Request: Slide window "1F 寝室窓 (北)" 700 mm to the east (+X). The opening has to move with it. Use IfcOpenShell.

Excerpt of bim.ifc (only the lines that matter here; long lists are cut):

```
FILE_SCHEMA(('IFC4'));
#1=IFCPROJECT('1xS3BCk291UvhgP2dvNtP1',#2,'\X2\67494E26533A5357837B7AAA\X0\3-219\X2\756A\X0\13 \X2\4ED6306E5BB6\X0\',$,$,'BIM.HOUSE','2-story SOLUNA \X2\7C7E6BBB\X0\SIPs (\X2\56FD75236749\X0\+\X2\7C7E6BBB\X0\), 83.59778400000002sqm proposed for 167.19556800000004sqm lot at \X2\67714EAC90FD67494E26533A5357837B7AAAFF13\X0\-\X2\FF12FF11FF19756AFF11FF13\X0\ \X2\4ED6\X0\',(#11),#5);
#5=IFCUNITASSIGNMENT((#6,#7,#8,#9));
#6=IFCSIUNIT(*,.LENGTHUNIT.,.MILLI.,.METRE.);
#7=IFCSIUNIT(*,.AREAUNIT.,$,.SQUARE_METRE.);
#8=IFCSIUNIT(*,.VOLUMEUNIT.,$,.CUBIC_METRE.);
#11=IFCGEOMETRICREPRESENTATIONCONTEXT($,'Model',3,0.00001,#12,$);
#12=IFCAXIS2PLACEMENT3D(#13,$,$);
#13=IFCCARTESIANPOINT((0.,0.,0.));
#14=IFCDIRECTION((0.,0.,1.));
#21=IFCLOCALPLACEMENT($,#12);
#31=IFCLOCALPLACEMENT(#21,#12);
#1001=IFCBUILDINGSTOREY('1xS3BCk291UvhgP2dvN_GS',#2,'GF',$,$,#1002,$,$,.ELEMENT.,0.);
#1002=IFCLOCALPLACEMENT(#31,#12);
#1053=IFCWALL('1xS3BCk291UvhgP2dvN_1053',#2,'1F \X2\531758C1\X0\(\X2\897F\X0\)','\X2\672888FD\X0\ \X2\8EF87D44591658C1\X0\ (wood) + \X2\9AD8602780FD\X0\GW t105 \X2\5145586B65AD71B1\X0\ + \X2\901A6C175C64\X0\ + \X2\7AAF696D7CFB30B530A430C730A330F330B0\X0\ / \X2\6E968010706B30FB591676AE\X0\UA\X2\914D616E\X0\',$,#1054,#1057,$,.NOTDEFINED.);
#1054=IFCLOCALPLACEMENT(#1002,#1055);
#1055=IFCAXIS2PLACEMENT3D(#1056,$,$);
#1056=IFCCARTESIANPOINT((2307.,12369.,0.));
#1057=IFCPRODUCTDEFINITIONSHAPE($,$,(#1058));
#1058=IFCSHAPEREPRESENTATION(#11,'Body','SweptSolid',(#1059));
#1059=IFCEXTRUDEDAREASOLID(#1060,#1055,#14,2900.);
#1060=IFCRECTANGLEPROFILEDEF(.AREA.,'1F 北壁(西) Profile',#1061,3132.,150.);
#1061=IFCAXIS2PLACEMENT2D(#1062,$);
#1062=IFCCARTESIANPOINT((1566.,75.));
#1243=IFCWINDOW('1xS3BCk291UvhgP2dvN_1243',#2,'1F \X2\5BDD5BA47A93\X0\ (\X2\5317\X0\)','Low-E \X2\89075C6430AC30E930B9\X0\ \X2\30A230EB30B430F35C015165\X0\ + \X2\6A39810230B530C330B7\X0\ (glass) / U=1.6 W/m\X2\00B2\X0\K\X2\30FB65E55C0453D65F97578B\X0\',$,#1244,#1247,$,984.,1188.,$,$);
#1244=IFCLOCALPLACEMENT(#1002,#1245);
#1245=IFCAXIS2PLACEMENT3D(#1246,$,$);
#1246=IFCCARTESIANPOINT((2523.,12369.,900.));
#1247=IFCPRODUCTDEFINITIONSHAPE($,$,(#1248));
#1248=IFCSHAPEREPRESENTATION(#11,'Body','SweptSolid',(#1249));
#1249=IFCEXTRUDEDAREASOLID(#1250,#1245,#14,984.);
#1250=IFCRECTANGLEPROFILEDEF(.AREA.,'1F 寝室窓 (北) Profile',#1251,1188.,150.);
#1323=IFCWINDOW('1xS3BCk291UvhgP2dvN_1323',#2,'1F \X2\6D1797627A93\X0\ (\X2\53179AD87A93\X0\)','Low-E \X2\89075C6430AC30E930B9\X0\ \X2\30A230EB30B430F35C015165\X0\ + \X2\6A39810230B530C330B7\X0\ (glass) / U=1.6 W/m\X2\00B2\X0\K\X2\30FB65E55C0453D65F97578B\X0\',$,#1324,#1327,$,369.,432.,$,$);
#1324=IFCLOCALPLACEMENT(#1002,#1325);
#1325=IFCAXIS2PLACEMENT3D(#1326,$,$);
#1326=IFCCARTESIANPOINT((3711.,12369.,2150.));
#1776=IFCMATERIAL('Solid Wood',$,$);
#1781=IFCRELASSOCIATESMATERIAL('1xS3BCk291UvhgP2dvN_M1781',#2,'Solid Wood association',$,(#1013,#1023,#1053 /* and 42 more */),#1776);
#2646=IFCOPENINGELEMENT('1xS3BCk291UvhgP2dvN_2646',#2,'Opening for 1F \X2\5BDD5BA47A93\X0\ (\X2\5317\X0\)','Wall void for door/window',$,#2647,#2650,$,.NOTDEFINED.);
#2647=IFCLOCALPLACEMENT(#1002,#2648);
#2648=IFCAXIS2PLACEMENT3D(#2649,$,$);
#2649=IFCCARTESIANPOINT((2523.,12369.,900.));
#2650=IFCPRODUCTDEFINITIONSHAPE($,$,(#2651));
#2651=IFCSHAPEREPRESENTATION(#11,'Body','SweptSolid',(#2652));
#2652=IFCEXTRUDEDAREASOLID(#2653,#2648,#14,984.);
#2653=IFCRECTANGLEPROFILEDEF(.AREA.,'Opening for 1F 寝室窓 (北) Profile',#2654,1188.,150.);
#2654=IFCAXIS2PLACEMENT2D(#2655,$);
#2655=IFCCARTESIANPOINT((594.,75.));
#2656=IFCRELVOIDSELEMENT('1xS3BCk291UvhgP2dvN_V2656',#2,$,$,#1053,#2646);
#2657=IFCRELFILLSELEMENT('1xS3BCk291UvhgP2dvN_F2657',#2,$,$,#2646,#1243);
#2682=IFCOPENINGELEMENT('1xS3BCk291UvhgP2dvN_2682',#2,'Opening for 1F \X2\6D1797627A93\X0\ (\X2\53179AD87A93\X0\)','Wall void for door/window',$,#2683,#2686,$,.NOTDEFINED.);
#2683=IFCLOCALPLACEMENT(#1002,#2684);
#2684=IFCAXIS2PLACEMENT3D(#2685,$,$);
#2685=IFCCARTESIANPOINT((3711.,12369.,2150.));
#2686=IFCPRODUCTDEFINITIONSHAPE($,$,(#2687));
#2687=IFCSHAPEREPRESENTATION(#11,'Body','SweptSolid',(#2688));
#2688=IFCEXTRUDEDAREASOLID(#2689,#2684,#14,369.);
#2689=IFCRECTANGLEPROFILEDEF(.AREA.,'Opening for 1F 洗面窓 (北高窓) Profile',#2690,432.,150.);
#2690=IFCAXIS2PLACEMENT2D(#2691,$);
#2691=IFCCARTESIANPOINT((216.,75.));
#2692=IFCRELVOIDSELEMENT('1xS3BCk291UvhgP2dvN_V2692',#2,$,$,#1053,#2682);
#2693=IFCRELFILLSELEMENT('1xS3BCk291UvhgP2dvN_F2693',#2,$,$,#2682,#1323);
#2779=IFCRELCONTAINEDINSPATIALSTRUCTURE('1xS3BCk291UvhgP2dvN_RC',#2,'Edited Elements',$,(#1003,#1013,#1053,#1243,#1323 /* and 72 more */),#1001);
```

```python
import ifcopenshell
import ifcopenshell.api.geometry
import ifcopenshell.util.placement
import ifcopenshell.util.unit

model = ifcopenshell.open("bim.ifc")
unit_scale = ifcopenshell.util.unit.calculate_unit_scale(model)

window = model.by_id(1243)
opening = window.FillsVoids[0].RelatingOpeningElement
wall = opening.VoidsElements[0].RelatingBuildingElement

wall_matrix = ifcopenshell.util.placement.get_local_placement(wall.ObjectPlacement)
shift = wall_matrix[:3, 0] * 0.7 / unit_scale
before = ifcopenshell.util.placement.get_local_placement(window.ObjectPlacement)[:3, 3].copy()

# The window is not placed relative to its opening, so move both.
for product in (opening, window):
    matrix = ifcopenshell.util.placement.get_local_placement(product.ObjectPlacement)
    matrix[:3, 3] += shift
    ifcopenshell.api.geometry.edit_object_placement(model, product=product, matrix=matrix, is_si=False)

after = ifcopenshell.util.placement.get_local_placement(window.ObjectPlacement)[:3, 3]
print("window moved by", (after - before).round(3) + 0.0)

model.write("bim_v2.ifc")
```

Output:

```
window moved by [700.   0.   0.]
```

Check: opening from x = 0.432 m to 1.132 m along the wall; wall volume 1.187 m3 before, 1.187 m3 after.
